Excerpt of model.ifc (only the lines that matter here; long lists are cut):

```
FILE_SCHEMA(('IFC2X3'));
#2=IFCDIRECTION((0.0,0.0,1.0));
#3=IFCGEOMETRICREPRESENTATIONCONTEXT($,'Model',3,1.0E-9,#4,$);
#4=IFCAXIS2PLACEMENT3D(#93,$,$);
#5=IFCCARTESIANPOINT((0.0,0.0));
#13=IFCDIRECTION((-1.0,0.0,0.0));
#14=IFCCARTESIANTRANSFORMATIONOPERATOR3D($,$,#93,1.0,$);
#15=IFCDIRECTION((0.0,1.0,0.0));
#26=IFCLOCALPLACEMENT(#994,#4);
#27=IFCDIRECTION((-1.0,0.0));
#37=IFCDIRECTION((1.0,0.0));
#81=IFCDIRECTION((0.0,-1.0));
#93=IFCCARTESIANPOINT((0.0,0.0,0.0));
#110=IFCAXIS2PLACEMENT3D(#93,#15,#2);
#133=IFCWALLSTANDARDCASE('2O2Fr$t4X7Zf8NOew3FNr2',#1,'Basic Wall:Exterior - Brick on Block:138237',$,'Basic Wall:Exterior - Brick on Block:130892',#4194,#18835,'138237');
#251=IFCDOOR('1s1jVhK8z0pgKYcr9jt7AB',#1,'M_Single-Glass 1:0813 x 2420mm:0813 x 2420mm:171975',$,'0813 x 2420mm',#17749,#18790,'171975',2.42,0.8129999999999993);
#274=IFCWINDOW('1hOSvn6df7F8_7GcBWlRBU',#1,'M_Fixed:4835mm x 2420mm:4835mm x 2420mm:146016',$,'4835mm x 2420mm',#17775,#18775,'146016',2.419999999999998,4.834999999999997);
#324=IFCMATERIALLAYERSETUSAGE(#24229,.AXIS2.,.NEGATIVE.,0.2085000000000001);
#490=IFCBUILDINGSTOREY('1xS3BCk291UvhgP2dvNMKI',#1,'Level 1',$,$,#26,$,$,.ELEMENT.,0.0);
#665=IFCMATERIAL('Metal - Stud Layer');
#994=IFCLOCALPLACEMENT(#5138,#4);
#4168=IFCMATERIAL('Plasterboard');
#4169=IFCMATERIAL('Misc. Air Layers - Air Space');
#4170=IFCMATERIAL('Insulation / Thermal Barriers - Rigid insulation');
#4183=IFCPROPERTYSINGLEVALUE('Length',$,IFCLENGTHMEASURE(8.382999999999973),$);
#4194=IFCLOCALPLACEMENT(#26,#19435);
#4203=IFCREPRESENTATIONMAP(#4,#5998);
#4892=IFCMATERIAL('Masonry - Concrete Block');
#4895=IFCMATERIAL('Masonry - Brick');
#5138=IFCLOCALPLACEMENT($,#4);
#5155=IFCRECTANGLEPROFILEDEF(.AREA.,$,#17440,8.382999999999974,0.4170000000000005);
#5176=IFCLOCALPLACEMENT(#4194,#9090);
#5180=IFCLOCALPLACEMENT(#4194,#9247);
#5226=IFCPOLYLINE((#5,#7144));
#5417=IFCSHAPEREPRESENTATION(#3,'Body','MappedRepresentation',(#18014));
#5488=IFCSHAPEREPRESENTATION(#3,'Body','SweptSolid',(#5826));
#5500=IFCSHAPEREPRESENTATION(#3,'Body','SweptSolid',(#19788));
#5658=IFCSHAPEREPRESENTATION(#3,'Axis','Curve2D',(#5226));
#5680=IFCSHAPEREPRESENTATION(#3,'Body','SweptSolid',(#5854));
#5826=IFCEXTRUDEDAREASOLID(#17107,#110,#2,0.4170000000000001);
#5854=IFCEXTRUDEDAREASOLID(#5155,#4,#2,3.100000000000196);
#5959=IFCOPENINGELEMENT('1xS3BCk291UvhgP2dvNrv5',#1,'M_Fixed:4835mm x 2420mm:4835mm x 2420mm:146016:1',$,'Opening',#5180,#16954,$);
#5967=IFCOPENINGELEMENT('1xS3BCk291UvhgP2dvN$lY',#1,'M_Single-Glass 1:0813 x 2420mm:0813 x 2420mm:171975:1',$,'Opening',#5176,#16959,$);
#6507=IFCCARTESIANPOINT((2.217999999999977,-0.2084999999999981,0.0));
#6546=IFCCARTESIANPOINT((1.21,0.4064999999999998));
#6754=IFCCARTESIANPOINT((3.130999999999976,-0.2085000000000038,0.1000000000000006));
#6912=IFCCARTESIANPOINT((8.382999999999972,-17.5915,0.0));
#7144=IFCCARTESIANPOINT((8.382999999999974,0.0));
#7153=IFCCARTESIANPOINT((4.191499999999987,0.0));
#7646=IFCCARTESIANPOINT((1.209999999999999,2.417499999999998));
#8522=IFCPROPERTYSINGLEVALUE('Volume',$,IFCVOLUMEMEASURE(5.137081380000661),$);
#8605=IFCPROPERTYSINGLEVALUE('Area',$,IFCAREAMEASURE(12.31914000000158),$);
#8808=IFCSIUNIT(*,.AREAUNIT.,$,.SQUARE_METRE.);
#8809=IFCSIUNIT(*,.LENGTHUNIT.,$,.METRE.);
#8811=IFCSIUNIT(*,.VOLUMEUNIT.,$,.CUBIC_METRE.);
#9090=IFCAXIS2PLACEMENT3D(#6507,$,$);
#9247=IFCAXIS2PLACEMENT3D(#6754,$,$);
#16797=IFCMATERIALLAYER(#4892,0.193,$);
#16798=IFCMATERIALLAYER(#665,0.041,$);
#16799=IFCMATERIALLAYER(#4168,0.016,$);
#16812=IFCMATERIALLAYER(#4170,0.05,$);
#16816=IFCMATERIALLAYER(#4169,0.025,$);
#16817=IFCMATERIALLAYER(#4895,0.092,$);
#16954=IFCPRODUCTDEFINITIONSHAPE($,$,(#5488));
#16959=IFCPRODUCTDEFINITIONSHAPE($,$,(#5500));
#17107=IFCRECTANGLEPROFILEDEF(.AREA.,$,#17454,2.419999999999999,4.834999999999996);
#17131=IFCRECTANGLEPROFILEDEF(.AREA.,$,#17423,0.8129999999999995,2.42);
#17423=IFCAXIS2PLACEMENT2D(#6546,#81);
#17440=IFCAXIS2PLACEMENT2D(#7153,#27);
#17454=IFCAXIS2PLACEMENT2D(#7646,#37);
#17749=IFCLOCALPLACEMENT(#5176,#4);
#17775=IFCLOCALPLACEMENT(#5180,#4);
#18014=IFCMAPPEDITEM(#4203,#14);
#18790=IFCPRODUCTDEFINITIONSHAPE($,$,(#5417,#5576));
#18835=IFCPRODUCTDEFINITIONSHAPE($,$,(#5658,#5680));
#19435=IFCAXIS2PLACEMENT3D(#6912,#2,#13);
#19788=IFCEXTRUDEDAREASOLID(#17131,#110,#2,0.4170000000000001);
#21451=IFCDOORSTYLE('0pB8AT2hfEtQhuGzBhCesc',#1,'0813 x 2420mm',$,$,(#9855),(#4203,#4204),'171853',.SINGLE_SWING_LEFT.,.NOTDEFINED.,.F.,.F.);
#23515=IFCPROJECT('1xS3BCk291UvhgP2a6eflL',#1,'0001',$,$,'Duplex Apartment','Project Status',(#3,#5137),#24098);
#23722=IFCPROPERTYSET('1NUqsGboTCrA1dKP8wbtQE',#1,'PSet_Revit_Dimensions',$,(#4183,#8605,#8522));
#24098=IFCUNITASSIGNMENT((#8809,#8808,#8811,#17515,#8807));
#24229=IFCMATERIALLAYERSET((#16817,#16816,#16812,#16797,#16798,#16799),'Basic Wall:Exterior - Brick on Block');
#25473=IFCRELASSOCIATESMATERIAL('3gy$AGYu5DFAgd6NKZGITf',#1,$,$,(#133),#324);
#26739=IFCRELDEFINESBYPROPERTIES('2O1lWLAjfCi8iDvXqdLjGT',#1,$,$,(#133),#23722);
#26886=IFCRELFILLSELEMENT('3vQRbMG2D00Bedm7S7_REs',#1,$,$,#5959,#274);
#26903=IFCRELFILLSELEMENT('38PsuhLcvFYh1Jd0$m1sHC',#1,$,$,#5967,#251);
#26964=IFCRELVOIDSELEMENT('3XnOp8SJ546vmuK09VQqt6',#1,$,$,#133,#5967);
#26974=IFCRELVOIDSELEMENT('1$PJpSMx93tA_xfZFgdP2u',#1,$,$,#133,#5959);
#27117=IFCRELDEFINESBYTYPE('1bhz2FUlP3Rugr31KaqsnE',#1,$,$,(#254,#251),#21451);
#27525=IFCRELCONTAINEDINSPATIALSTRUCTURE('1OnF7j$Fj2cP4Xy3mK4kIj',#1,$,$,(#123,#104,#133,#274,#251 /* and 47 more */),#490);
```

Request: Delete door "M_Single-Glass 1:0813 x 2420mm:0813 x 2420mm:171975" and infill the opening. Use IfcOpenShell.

```python
import ifcopenshell
import ifcopenshell.api.feature
import ifcopenshell.api.pset
import ifcopenshell.api.root
import ifcopenshell.geom
import ifcopenshell.util.element
import ifcopenshell.util.shape
import ifcopenshell.util.unit

model = ifcopenshell.open("model.ifc")
area_scale = ifcopenshell.util.unit.calculate_unit_scale(model, "AREAUNIT")
volume_scale = ifcopenshell.util.unit.calculate_unit_scale(model, "VOLUMEUNIT")
settings = ifcopenshell.geom.settings()


def volume(element):
    """Net volume in cubic metres, openings subtracted."""
    shape = ifcopenshell.geom.create_shape(settings, element)
    return ifcopenshell.util.shape.get_volume(shape.geometry)


door = model.by_guid("1s1jVhK8z0pgKYcr9jt7AB")
opening = door.FillsVoids[0].RelatingOpeningElement
wall = opening.VoidsElements[0].RelatingBuildingElement
before = volume(wall)

ifcopenshell.api.root.remove_product(model, product=door)
ifcopenshell.api.feature.remove_feature(model, feature=opening)

after = volume(wall)
thickness = 0.417  # wall thickness in metres

# Update the wall's stored quantities.
pset = model.by_id(ifcopenshell.util.element.get_pset(wall, "PSet_Revit_Dimensions", should_inherit=False)["id"])
ifcopenshell.api.pset.edit_pset(model, pset=pset, properties={
    "Area": model.create_entity("IfcAreaMeasure", after / thickness / area_scale),
    "Volume": model.create_entity("IfcVolumeMeasure", after / volume_scale),
})

print(f"wall volume {before:.3f} -> {after:.3f} m3")

model.write("model_updated.ifc")
```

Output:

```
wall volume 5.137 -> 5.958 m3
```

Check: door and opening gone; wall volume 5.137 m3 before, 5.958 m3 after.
